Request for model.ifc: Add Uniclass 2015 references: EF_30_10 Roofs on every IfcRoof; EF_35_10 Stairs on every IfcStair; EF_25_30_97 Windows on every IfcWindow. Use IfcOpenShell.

First a look at what the model holds.

```python
import ifcopenshell

model = ifcopenshell.open("model.ifc")
print(model.schema)
print("classifications:", [c.Name for c in model.by_type("IfcClassification")])
for ifc_class in ("IfcDoor", "IfcRoof", "IfcStair", "IfcWall", "IfcWindow"):
    print(ifc_class, len(model.by_type(ifc_class)))
```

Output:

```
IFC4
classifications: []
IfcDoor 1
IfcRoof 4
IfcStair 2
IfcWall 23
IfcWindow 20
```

```python
import ifcopenshell
import ifcopenshell.api.classification

model = ifcopenshell.open("model.ifc")

system = ifcopenshell.api.classification.add_classification(model, classification="Uniclass 2015")

codes = {
    "IfcRoof": ("EF_30_10", "Roofs"),
    "IfcStair": ("EF_35_10", "Stairs"),
    "IfcWindow": ("EF_25_30_97", "Windows"),
}
for ifc_class, (code, name) in codes.items():
    products = model.by_type(ifc_class)
    ifcopenshell.api.classification.add_reference(
        model, products=products, classification=system, identification=code, name=name
    )
    print(code, len(products))

model.write("model_v2.ifc")
```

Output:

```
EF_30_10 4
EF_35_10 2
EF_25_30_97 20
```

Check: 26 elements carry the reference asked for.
